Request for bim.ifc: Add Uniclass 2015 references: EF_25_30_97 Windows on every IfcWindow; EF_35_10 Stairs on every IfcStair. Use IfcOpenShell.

First a look at what the model holds.

```python
import ifcopenshell

model = ifcopenshell.open("bim.ifc")
print(model.schema)
print("classifications:", [c.Name for c in model.by_type("IfcClassification")])
for ifc_class in ("IfcDoor", "IfcRoof", "IfcStair", "IfcWall", "IfcWindow"):
    print(ifc_class, len(model.by_type(ifc_class)))
```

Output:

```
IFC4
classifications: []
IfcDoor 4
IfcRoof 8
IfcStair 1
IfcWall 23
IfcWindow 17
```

```python
import ifcopenshell
import ifcopenshell.api.classification

model = ifcopenshell.open("bim.ifc")

system = ifcopenshell.api.classification.add_classification(model, classification="Uniclass 2015")

codes = {
    "IfcWindow": ("EF_25_30_97", "Windows"),
    "IfcStair": ("EF_35_10", "Stairs"),
}
for ifc_class, (code, name) in codes.items():
    products = model.by_type(ifc_class)
    ifcopenshell.api.classification.add_reference(
        model, products=products, classification=system, identification=code, name=name
    )
    print(code, len(products))

model.write("bim_v2.ifc")
```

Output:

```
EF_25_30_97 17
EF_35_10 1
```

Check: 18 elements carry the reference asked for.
